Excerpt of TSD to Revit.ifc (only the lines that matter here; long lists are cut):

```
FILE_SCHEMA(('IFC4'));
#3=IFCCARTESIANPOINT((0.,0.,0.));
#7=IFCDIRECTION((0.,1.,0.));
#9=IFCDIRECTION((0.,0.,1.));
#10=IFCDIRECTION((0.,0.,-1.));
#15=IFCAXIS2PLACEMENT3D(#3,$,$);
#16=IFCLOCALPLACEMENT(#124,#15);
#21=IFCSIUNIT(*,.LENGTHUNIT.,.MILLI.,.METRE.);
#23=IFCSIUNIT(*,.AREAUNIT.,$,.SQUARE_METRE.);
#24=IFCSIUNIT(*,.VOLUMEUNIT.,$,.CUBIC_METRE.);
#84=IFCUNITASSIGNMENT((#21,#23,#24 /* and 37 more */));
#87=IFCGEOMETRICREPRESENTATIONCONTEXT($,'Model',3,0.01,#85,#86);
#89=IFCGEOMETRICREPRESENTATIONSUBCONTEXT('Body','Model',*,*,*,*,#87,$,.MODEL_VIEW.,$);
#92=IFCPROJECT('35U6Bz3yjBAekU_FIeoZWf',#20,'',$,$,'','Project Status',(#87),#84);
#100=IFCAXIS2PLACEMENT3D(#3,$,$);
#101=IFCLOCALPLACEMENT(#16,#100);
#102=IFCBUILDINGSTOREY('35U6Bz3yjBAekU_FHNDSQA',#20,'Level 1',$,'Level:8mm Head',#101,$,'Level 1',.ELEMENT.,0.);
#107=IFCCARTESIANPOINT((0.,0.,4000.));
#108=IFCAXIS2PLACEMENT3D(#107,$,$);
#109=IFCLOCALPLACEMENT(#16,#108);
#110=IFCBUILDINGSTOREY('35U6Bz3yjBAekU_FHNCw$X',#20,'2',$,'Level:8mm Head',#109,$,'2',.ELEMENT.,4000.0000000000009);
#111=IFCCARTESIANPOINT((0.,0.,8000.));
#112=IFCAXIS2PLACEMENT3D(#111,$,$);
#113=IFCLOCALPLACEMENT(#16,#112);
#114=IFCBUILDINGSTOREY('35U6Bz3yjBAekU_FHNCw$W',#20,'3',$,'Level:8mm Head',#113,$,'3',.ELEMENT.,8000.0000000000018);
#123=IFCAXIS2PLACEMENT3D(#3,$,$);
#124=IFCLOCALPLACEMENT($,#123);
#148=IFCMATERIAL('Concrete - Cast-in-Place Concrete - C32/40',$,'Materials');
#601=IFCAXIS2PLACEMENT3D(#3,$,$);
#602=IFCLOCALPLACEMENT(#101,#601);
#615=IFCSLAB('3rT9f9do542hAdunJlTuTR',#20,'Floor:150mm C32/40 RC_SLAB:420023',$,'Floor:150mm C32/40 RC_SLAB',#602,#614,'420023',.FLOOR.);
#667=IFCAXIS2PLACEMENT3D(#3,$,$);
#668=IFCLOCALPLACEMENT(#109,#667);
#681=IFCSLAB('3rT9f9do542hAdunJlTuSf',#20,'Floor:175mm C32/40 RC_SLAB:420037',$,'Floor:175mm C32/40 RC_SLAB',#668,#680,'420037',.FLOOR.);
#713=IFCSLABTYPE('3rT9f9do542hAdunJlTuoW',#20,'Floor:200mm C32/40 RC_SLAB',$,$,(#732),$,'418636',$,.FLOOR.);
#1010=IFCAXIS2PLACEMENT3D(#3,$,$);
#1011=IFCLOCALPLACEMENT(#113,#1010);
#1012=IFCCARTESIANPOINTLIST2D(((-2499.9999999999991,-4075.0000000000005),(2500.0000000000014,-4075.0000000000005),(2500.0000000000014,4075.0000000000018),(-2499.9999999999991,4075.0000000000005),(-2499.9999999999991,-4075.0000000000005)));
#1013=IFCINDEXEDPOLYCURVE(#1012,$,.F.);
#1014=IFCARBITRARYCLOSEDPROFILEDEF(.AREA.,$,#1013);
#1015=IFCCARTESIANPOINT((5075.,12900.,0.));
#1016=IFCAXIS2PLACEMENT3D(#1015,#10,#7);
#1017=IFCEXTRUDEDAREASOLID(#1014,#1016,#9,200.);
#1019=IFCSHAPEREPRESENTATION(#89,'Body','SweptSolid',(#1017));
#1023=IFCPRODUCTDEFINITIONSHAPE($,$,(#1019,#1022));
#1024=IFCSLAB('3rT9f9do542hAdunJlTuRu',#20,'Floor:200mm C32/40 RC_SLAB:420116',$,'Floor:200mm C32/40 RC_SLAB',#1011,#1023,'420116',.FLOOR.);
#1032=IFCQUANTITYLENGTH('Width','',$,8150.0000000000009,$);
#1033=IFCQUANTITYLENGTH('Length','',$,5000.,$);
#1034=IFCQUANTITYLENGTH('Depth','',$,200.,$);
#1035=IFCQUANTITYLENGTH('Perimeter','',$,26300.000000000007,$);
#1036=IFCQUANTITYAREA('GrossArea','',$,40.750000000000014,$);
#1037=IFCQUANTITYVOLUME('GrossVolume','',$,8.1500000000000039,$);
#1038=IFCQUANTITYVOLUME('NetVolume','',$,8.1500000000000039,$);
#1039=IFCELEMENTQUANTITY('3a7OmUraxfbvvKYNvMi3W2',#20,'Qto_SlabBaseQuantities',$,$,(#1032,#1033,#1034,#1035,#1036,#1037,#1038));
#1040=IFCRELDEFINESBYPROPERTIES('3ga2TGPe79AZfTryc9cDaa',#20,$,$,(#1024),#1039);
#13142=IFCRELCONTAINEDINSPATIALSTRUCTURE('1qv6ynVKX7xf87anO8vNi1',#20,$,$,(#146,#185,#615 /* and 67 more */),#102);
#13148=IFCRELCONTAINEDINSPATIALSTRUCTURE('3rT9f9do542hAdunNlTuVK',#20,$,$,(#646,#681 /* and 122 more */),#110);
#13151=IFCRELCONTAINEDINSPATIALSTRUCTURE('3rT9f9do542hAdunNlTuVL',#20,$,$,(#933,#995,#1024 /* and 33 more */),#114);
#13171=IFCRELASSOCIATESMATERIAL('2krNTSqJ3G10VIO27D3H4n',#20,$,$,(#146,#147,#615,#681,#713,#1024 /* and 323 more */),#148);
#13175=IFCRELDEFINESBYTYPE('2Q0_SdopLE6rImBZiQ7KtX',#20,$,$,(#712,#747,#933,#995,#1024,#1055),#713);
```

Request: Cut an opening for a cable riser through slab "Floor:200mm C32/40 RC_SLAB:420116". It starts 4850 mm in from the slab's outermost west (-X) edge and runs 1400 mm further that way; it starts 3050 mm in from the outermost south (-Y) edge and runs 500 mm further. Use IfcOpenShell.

```python
import numpy as np
import ifcopenshell
import ifcopenshell.api.feature
import ifcopenshell.api.geometry
import ifcopenshell.api.pset
import ifcopenshell.api.root
import ifcopenshell.geom
import ifcopenshell.util.element
import ifcopenshell.util.placement
import ifcopenshell.util.representation
import ifcopenshell.util.shape
import ifcopenshell.util.unit

model = ifcopenshell.open("TSD to Revit.ifc")
unit_scale = ifcopenshell.util.unit.calculate_unit_scale(model)
volume_scale = ifcopenshell.util.unit.calculate_unit_scale(model, "VOLUMEUNIT")
settings = ifcopenshell.geom.settings()


def volume(element):
    """Net volume in cubic metres, openings subtracted."""
    shape = ifcopenshell.geom.create_shape(settings, element)
    return ifcopenshell.util.shape.get_volume(shape.geometry)


slab = model.by_guid("3rT9f9do542hAdunJlTuRu")
before = volume(slab)

# Extent in the slab's own axes, in metres. The edges named are its -X and -Y sides.
slab_shape = ifcopenshell.geom.create_shape(settings, slab)
vertices = ifcopenshell.util.shape.get_vertices(slab_shape.geometry)
x_min, y_min, bottom = vertices.min(axis=0)
top = vertices[:, 2].max()

opening = ifcopenshell.api.root.create_entity(model, ifc_class="IfcOpeningElement", name="Cable riser opening", predefined_type="OPENING")
context = ifcopenshell.util.representation.get_context(model, "Model", "Body", "MODEL_VIEW")
width, depth = 1.4, 0.5
outline = [(0.0, 0.0), (width, 0.0), (width, depth), (0.0, depth), (0.0, 0.0)]
# Overshoot both faces by 50 mm so the cut is clean.
shape = ifcopenshell.api.geometry.add_slab_representation(
    model, context=context, depth=top - bottom + 0.1, polyline=outline
)
ifcopenshell.api.geometry.assign_representation(model, product=opening, representation=shape)

matrix = ifcopenshell.util.placement.get_local_placement(slab.ObjectPlacement)
matrix[:, 3] = matrix @ np.append(np.array([x_min + 4.85, y_min + 3.05, bottom - 0.05]) / unit_scale, 1.0)
ifcopenshell.api.geometry.edit_object_placement(model, product=opening, matrix=matrix, is_si=False)
ifcopenshell.api.feature.add_feature(model, feature=opening, element=slab)

after = volume(slab)

# Update the slab's stored quantities.
qto = model.by_id(ifcopenshell.util.element.get_pset(slab, "Qto_SlabBaseQuantities", should_inherit=False)["id"])
ifcopenshell.api.pset.edit_qto(model, qto=qto, properties={"NetVolume": after / volume_scale})

print(f"slab volume {before:.3f} -> {after:.3f} m3")

model.write("TSD to Revit_edited.ifc")
```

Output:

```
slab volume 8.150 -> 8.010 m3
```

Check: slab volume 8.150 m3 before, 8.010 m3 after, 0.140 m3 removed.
